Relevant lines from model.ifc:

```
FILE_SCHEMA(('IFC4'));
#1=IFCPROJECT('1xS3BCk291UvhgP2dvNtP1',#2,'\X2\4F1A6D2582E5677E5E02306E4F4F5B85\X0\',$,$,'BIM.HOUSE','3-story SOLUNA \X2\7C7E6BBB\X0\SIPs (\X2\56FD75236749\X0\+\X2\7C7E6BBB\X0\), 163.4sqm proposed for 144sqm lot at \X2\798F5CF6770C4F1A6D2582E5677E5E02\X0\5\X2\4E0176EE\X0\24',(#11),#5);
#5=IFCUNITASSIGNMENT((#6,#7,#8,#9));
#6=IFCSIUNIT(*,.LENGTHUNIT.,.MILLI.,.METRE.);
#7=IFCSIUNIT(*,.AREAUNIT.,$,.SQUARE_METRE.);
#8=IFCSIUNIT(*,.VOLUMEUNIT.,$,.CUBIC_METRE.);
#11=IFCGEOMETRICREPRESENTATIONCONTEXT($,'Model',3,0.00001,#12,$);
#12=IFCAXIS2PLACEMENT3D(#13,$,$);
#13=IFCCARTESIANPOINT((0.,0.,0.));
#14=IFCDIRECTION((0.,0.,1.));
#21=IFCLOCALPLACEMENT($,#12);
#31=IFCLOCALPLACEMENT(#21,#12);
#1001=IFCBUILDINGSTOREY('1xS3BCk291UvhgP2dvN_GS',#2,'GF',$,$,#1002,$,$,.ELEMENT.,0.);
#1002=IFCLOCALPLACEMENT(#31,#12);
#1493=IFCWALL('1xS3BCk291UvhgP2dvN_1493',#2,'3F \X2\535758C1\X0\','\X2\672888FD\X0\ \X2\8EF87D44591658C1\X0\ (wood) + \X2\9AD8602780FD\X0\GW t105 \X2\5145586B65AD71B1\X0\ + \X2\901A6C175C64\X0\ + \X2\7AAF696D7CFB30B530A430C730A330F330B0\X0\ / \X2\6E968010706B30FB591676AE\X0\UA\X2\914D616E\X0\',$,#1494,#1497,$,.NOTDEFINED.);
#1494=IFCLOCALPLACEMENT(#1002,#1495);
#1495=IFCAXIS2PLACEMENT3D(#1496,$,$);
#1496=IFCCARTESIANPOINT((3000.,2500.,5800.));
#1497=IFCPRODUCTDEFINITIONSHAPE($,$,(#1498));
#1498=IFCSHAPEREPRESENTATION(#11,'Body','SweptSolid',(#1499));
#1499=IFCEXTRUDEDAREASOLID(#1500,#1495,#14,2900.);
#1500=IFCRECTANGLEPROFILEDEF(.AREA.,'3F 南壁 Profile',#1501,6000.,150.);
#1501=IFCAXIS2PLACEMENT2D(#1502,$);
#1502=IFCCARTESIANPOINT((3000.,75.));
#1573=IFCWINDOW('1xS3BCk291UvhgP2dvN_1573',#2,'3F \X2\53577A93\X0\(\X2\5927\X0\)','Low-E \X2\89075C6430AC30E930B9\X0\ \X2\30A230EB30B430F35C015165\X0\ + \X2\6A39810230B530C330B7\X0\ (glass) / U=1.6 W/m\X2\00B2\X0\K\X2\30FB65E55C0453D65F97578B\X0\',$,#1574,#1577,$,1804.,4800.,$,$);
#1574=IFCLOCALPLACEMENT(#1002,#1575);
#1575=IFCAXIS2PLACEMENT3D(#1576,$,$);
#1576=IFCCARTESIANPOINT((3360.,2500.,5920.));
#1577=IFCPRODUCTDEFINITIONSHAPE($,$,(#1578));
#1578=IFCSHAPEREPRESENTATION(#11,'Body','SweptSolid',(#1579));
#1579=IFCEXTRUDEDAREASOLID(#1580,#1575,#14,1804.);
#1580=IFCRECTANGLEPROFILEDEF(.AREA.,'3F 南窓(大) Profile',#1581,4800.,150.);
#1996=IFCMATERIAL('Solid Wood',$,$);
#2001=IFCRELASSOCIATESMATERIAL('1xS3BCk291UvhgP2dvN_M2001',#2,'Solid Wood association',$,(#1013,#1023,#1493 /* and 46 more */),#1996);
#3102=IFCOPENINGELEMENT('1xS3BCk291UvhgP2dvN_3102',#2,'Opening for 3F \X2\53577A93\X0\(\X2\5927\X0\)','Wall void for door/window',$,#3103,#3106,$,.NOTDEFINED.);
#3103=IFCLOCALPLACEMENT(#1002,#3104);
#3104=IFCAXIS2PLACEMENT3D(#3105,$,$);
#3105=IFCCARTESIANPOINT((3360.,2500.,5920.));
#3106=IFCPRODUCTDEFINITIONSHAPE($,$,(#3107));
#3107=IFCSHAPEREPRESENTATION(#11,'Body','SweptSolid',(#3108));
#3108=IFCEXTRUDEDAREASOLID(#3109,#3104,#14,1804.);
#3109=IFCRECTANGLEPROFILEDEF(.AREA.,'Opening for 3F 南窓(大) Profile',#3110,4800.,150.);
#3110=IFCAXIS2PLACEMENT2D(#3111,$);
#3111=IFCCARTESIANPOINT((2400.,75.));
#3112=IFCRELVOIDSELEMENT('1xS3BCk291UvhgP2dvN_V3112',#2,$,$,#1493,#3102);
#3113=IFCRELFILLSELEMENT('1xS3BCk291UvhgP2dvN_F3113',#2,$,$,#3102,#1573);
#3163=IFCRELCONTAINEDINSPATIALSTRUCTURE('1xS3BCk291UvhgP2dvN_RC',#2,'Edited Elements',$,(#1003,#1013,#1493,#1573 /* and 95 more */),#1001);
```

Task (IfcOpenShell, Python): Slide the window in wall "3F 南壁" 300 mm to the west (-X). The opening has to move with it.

```python
import ifcopenshell
import ifcopenshell.api.geometry
import ifcopenshell.util.placement

model = ifcopenshell.open("model.ifc")

window = model.by_guid("1xS3BCk291UvhgP2dvN_1573")
opening = window.FillsVoids[0].RelatingOpeningElement
wall = opening.VoidsElements[0].RelatingBuildingElement

wall_matrix = ifcopenshell.util.placement.get_local_placement(wall.ObjectPlacement)
shift = wall_matrix[:3, 0] * -300.0
before = ifcopenshell.util.placement.get_local_placement(window.ObjectPlacement)[:3, 3].copy()

# The window is not placed relative to its opening, so move both.
for product in (opening, window):
    matrix = ifcopenshell.util.placement.get_local_placement(product.ObjectPlacement)
    matrix[:3, 3] += shift
    ifcopenshell.api.geometry.edit_object_placement(model, product=product, matrix=matrix, is_si=False)

after = ifcopenshell.util.placement.get_local_placement(window.ObjectPlacement)[:3, 3]
print("window moved by", (after - before).round(3) + 0.0)

model.write("model_updated.ifc")
```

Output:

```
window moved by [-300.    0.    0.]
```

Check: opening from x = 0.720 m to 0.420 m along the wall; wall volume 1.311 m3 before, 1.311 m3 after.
